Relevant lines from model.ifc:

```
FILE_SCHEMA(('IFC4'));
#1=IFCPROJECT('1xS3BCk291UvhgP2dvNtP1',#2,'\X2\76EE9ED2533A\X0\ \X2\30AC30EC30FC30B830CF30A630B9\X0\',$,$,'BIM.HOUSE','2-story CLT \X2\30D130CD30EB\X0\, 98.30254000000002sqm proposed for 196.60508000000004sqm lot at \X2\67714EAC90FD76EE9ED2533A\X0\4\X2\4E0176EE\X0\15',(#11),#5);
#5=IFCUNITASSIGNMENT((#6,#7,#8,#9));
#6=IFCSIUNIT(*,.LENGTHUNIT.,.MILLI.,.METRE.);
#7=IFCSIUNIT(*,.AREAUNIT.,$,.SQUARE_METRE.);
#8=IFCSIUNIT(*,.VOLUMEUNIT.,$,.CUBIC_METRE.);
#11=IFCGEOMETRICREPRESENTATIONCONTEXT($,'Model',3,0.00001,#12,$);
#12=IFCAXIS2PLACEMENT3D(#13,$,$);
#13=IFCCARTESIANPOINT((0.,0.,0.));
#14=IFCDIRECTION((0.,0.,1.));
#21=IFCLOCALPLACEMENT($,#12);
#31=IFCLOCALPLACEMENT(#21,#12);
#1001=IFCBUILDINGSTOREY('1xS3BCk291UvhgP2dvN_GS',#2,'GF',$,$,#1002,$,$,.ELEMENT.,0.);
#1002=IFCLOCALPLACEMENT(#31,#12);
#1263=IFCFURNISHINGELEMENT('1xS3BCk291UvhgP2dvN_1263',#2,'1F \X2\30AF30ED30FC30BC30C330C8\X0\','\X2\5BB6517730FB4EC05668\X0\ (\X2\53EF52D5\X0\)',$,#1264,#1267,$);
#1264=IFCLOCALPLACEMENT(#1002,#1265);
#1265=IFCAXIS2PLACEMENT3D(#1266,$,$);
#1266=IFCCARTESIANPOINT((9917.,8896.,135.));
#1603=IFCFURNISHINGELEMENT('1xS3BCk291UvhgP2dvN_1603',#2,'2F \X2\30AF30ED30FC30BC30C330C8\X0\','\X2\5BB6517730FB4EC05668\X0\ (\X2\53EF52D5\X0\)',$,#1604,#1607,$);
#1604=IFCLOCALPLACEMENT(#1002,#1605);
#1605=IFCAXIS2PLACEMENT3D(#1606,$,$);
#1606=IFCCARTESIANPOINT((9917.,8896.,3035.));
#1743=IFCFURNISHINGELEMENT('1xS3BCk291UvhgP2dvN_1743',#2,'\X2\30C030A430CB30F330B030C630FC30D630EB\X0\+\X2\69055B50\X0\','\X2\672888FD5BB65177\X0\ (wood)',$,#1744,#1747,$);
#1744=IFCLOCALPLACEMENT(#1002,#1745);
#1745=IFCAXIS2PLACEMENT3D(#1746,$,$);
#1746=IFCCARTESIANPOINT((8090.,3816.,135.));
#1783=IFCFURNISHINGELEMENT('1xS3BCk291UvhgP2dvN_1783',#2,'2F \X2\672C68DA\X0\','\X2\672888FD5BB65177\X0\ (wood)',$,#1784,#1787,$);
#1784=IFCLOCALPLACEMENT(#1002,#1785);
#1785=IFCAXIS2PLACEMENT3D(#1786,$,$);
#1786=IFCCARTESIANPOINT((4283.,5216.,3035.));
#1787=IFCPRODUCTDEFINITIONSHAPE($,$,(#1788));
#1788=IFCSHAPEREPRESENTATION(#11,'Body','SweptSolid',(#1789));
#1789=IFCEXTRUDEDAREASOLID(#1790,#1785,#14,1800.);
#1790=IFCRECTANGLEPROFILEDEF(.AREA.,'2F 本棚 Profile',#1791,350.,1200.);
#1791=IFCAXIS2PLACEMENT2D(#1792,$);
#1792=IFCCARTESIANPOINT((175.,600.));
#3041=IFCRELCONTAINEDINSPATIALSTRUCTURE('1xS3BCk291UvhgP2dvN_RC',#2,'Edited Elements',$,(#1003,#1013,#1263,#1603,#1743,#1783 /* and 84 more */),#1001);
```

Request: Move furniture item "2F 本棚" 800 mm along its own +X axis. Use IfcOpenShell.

```python
import ifcopenshell
import ifcopenshell.api.geometry
import ifcopenshell.util.placement

model = ifcopenshell.open("model.ifc")

item = model.by_guid("1xS3BCk291UvhgP2dvN_1783")
matrix = ifcopenshell.util.placement.get_local_placement(item.ObjectPlacement)
matrix[:3, 3] += matrix[:3, 0] * 800.0
ifcopenshell.api.geometry.edit_object_placement(model, product=item, matrix=matrix, is_si=False)

print(ifcopenshell.util.placement.get_local_placement(item.ObjectPlacement).round(3) + 0.0)

model.write("model_rev.ifc")
```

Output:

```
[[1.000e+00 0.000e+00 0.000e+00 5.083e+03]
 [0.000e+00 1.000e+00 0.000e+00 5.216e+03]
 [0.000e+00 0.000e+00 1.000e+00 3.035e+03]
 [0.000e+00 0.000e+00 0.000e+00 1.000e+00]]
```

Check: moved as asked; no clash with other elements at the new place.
